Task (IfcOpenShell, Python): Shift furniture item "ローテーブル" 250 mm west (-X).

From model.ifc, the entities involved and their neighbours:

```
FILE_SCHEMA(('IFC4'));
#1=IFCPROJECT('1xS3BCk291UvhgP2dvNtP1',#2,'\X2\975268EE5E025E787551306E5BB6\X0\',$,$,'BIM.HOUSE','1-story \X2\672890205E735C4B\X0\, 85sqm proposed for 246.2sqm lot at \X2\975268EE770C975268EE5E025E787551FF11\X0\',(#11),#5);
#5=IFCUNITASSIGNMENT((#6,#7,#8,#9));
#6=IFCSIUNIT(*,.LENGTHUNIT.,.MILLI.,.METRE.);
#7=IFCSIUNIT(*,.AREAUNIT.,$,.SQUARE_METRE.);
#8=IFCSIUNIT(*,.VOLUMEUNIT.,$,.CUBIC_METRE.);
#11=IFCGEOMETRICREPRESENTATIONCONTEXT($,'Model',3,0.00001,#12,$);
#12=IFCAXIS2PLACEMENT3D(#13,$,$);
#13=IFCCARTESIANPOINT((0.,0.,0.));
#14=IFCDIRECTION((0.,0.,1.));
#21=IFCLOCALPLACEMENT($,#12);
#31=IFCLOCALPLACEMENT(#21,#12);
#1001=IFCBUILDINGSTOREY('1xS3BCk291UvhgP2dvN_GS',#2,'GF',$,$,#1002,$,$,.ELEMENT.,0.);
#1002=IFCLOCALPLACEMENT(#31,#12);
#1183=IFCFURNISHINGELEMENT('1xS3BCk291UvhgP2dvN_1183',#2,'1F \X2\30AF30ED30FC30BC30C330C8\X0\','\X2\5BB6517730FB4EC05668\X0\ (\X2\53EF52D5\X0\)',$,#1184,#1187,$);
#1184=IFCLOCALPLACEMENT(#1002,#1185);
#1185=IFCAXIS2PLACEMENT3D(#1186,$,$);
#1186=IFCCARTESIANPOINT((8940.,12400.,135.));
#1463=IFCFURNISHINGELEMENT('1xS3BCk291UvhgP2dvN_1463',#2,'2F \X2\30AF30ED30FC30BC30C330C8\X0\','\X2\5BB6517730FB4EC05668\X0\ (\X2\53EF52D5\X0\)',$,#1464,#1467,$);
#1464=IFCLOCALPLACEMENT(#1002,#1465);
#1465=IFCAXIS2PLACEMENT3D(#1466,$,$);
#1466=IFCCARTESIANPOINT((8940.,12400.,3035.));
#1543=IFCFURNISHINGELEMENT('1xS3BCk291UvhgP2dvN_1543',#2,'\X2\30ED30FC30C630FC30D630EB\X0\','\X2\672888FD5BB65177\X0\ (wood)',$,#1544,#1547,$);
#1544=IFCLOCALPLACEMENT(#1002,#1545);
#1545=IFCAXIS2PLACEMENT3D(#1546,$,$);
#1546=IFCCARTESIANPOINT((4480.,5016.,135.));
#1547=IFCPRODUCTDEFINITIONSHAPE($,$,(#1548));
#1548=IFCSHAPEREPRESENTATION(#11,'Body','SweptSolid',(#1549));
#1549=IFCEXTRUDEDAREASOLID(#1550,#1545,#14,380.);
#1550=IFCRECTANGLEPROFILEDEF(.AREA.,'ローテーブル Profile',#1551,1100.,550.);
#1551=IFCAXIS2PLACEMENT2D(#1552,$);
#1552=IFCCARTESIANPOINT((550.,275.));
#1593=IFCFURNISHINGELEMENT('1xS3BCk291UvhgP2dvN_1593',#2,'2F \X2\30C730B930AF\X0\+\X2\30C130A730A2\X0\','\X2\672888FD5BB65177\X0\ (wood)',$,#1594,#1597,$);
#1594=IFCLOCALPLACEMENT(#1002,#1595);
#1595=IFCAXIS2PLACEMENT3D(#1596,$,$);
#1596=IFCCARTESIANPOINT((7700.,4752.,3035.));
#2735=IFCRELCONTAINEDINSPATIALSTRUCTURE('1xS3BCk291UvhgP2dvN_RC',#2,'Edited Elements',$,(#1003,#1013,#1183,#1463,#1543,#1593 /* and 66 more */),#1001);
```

```python
import ifcopenshell
import ifcopenshell.api.geometry
import ifcopenshell.util.placement
import ifcopenshell.util.unit

model = ifcopenshell.open("model.ifc")
unit_scale = ifcopenshell.util.unit.calculate_unit_scale(model)

item = model.by_id(1543)
matrix = ifcopenshell.util.placement.get_local_placement(item.ObjectPlacement)
matrix[0, 3] -= 0.25 / unit_scale
ifcopenshell.api.geometry.edit_object_placement(model, product=item, matrix=matrix, is_si=False)

print(ifcopenshell.util.placement.get_local_placement(item.ObjectPlacement).round(3) + 0.0)

model.write("model_rev.ifc")
```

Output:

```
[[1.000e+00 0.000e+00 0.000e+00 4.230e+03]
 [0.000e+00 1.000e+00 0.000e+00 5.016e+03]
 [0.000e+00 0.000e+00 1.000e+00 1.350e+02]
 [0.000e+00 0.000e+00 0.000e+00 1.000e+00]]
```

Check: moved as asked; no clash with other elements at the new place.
